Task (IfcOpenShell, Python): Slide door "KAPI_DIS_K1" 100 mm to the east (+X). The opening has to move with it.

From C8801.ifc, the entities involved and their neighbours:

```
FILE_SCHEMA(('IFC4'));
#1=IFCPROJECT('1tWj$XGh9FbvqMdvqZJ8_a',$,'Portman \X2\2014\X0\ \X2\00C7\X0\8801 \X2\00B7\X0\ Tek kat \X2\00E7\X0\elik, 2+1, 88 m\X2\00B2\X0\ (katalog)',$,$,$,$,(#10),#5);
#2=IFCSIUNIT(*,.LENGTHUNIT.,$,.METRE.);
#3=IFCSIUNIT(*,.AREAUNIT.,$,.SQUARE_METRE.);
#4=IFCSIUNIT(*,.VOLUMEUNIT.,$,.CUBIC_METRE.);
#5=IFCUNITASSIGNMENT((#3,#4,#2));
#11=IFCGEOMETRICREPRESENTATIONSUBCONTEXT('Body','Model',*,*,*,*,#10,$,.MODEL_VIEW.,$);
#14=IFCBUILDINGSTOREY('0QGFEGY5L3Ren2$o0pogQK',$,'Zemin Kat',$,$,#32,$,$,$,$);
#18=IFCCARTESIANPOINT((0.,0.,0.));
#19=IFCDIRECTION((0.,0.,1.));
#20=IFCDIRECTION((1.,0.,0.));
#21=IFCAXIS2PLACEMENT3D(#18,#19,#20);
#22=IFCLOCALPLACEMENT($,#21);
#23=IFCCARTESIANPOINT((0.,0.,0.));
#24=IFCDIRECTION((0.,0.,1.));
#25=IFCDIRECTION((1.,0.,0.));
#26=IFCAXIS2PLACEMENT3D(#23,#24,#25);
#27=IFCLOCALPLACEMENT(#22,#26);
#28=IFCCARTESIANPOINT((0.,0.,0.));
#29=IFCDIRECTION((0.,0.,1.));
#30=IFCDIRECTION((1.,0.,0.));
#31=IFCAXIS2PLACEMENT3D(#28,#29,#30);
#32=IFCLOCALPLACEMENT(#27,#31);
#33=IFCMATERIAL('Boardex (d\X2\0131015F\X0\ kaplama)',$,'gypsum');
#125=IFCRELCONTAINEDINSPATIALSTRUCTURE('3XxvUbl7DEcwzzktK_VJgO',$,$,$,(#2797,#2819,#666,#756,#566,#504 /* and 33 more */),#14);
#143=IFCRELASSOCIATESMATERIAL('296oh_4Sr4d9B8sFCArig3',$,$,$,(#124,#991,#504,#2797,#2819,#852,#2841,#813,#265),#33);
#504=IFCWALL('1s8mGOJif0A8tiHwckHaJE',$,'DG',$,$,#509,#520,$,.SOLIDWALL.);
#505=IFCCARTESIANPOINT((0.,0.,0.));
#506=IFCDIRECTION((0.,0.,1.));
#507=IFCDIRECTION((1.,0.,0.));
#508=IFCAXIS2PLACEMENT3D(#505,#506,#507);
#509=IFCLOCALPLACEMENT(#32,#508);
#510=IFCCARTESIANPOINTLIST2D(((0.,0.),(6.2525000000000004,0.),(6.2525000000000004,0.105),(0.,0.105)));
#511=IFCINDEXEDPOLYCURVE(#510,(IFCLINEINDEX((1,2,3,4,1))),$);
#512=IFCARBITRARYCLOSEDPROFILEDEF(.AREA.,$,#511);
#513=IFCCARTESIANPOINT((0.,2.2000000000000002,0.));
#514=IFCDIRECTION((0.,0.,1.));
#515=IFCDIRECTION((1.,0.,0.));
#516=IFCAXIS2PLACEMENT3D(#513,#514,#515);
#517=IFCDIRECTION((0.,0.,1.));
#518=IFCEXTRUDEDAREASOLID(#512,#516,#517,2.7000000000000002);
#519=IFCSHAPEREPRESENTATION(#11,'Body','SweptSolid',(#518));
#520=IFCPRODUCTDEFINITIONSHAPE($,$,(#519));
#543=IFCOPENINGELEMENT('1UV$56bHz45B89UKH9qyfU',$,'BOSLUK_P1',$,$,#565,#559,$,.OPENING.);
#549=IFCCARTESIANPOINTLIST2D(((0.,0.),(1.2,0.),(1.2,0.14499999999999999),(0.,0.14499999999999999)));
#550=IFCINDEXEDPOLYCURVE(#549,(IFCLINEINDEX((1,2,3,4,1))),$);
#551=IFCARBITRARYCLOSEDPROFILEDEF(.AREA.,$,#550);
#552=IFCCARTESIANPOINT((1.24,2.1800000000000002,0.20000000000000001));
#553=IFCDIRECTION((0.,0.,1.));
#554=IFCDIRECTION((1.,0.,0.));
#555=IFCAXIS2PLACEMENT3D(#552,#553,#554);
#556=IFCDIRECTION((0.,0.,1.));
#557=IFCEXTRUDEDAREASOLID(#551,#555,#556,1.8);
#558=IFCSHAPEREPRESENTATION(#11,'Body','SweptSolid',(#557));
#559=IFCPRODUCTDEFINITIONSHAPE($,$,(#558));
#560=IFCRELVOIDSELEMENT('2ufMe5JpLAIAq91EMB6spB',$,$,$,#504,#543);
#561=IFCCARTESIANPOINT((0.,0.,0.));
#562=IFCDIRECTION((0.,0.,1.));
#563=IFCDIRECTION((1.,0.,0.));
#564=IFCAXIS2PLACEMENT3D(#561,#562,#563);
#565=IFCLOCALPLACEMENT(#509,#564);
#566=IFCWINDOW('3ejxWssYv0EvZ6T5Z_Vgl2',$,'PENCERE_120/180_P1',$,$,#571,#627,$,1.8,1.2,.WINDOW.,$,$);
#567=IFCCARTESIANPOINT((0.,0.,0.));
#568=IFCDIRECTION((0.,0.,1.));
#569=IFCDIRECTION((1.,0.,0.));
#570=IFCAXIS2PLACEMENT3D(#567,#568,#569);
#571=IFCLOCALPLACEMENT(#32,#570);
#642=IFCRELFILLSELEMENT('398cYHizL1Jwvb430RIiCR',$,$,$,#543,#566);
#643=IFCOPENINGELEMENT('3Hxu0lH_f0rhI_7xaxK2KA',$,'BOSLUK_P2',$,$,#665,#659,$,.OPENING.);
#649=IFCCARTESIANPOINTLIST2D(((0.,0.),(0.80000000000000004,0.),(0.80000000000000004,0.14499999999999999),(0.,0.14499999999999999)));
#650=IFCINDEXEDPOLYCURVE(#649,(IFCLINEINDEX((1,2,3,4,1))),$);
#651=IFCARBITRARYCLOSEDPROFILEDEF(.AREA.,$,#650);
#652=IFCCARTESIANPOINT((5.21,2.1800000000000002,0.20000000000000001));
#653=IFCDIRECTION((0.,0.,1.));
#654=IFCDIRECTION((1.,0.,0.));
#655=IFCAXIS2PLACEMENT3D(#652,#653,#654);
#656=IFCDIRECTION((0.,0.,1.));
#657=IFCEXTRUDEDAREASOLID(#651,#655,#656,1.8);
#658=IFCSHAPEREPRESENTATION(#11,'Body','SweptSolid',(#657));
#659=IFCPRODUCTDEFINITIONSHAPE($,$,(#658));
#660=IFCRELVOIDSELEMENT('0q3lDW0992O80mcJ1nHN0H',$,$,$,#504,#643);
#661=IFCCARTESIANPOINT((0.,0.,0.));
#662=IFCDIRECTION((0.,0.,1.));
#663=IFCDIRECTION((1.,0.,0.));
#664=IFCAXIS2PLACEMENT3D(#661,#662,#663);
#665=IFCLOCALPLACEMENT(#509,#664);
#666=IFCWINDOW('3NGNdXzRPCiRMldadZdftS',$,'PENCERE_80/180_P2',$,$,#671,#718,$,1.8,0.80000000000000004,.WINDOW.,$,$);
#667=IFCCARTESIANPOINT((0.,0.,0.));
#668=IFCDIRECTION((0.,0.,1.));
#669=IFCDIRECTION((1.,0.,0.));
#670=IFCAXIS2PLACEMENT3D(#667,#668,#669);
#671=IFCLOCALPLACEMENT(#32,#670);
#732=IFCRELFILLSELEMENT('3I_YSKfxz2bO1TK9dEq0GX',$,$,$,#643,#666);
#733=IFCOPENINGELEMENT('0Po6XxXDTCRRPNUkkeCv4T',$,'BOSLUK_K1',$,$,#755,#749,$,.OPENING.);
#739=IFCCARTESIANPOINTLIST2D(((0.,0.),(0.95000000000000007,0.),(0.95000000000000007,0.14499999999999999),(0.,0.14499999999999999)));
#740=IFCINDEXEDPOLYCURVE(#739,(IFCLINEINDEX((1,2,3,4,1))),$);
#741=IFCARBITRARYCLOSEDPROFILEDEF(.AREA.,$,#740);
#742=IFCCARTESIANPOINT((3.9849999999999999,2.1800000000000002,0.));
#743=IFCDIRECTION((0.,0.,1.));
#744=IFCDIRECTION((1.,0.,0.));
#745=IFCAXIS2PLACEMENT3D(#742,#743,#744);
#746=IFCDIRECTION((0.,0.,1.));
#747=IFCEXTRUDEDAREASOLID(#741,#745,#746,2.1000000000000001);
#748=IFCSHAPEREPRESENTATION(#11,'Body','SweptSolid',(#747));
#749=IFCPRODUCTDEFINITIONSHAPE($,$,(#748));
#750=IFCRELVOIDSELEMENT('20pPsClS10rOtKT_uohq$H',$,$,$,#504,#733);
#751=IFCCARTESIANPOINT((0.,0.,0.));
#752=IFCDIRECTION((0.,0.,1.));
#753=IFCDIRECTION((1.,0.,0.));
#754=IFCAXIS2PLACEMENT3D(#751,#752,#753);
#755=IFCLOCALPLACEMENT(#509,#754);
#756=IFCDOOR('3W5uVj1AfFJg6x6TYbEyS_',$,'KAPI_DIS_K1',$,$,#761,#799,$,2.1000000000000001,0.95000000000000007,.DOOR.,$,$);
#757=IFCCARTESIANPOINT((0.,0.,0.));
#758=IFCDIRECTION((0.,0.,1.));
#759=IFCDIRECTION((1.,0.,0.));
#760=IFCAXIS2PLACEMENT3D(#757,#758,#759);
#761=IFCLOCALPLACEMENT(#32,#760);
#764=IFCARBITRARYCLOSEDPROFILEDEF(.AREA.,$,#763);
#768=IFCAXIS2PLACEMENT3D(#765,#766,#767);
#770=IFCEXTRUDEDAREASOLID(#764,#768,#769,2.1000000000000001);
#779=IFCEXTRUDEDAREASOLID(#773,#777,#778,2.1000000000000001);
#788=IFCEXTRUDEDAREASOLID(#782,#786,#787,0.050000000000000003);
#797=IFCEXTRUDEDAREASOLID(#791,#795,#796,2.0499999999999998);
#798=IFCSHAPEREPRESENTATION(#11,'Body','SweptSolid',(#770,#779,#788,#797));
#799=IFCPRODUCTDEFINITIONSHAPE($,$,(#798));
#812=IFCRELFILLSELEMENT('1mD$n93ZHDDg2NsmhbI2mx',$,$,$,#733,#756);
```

```python
import ifcopenshell
import ifcopenshell.api.geometry
import ifcopenshell.util.placement
import ifcopenshell.util.unit

model = ifcopenshell.open("C8801.ifc")
unit_scale = ifcopenshell.util.unit.calculate_unit_scale(model)

door = model.by_id(756)
opening = door.FillsVoids[0].RelatingOpeningElement
wall = opening.VoidsElements[0].RelatingBuildingElement

wall_matrix = ifcopenshell.util.placement.get_local_placement(wall.ObjectPlacement)
shift = wall_matrix[:3, 0] * 0.1 / unit_scale
before = ifcopenshell.util.placement.get_local_placement(door.ObjectPlacement)[:3, 3].copy()

# The door is not placed relative to its opening, so move both.
for product in (opening, door):
    matrix = ifcopenshell.util.placement.get_local_placement(product.ObjectPlacement)
    matrix[:3, 3] += shift
    ifcopenshell.api.geometry.edit_object_placement(model, product=product, matrix=matrix, is_si=False)

after = ifcopenshell.util.placement.get_local_placement(door.ObjectPlacement)[:3, 3]
print("door moved by", (after - before).round(3) + 0.0)

model.write("C8801_edited.ifc")
```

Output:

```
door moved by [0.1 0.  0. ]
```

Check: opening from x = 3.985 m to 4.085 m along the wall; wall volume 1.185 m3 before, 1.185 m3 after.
